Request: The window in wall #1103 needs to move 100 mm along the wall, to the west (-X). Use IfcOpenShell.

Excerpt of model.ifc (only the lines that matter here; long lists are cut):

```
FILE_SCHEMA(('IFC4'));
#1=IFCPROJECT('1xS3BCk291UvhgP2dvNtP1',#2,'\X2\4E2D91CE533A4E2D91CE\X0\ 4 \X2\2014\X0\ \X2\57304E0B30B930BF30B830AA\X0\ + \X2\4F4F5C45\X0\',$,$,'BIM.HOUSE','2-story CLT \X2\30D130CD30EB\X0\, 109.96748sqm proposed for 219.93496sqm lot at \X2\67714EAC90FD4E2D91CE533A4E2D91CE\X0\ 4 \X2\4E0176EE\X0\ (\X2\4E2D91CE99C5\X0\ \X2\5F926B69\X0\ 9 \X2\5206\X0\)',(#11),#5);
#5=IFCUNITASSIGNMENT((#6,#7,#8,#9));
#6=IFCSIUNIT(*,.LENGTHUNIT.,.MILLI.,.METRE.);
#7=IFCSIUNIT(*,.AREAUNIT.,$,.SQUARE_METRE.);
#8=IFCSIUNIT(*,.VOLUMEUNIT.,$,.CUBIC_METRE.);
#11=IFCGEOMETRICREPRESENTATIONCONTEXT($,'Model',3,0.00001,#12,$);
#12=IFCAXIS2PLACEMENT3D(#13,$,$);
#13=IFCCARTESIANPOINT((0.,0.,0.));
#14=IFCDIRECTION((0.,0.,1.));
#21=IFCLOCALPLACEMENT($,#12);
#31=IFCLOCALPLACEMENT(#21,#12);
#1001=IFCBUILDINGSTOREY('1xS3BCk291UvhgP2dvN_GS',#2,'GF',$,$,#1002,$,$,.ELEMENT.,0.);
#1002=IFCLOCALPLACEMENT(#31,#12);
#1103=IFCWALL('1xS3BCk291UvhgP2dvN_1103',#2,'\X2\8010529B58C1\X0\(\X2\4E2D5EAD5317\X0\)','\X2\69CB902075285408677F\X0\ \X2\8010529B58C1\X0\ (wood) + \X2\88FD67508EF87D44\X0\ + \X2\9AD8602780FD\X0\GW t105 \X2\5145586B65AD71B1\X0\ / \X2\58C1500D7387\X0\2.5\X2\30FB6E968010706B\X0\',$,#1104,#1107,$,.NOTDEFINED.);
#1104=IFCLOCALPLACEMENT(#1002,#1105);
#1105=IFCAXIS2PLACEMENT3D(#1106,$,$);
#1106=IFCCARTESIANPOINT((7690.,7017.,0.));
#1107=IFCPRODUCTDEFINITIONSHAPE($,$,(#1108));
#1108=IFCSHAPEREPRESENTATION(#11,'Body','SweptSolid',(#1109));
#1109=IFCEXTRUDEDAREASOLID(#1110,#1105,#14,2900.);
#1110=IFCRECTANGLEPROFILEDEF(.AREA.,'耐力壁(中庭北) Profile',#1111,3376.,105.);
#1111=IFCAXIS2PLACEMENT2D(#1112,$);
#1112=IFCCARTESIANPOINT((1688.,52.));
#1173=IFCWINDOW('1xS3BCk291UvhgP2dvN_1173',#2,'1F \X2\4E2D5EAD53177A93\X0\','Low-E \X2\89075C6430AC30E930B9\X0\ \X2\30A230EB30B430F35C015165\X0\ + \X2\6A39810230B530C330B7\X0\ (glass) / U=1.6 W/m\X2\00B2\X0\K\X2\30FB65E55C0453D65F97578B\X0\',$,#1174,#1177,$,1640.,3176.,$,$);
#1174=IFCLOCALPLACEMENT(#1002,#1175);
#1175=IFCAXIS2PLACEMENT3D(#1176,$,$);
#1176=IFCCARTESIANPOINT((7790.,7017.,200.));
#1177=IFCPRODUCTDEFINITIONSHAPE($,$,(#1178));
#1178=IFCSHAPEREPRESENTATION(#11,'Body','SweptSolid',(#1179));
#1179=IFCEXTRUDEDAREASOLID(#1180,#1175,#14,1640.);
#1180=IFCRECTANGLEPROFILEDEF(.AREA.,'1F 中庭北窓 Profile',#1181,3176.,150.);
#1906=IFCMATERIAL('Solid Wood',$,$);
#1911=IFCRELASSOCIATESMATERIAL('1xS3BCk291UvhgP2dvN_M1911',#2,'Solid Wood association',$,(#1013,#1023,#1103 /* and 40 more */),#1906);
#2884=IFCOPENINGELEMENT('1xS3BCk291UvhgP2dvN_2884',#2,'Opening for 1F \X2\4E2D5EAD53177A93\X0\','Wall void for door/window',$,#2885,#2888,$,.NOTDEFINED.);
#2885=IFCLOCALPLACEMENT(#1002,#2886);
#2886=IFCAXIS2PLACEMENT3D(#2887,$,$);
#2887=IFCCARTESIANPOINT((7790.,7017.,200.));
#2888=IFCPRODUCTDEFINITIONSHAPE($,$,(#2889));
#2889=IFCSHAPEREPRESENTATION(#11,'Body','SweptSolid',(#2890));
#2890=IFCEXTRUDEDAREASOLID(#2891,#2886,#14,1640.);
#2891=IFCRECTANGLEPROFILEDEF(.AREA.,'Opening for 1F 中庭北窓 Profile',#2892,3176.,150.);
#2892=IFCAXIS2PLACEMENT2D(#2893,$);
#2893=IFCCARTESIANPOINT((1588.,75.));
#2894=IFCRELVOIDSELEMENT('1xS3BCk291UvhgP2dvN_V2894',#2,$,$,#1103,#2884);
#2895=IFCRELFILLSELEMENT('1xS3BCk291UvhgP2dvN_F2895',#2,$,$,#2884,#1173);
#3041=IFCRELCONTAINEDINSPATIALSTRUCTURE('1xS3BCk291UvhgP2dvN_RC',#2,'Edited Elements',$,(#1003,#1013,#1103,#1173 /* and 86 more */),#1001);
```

```python
import ifcopenshell
import ifcopenshell.api.geometry
import ifcopenshell.util.placement
import ifcopenshell.util.unit

model = ifcopenshell.open("model.ifc")
unit_scale = ifcopenshell.util.unit.calculate_unit_scale(model)

window = model.by_id(1173)
opening = window.FillsVoids[0].RelatingOpeningElement
wall = opening.VoidsElements[0].RelatingBuildingElement

wall_matrix = ifcopenshell.util.placement.get_local_placement(wall.ObjectPlacement)
shift = wall_matrix[:3, 0] * -0.1 / unit_scale
before = ifcopenshell.util.placement.get_local_placement(window.ObjectPlacement)[:3, 3].copy()

# The window is not placed relative to its opening, so move both.
for product in (opening, window):
    matrix = ifcopenshell.util.placement.get_local_placement(product.ObjectPlacement)
    matrix[:3, 3] += shift
    ifcopenshell.api.geometry.edit_object_placement(model, product=product, matrix=matrix, is_si=False)

after = ifcopenshell.util.placement.get_local_placement(window.ObjectPlacement)[:3, 3]
print("window moved by", (after - before).round(3) + 0.0)

model.write("model_rev.ifc")
```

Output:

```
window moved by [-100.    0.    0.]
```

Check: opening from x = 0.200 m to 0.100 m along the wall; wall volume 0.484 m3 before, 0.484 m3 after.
